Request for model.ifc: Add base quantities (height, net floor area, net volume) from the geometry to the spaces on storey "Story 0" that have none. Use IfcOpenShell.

First a look at what the model holds.

```python
import ifcopenshell
import ifcopenshell.util.element
import ifcopenshell.util.unit

model = ifcopenshell.open("model.ifc")
print(model.schema)
for unit_type in ("LENGTHUNIT", "AREAUNIT", "VOLUMEUNIT"):
    print(unit_type, ifcopenshell.util.unit.calculate_unit_scale(model, unit_type))
storey = next(s for s in model.by_type("IfcBuildingStorey") if s.Name == "Story 0")
spaces = [e for e in ifcopenshell.util.element.get_decomposition(storey) if e.is_a("IfcSpace")]
for e in sorted(spaces, key=lambda e: e.id()):
    print(e.id(), e.is_a(), e.Name, list(ifcopenshell.util.element.get_psets(e, qtos_only=True)), sep=" | ")
```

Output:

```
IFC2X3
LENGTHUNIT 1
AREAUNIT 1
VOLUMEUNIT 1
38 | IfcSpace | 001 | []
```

```python
import ifcopenshell
import ifcopenshell.api.pset
import ifcopenshell.geom
import ifcopenshell.util.element
import ifcopenshell.util.shape
import ifcopenshell.util.unit

model = ifcopenshell.open("model.ifc")
unit_scale = ifcopenshell.util.unit.calculate_unit_scale(model)
area_scale = ifcopenshell.util.unit.calculate_unit_scale(model, "AREAUNIT")
volume_scale = ifcopenshell.util.unit.calculate_unit_scale(model, "VOLUMEUNIT")
settings = ifcopenshell.geom.settings()

storey = next(s for s in model.by_type("IfcBuildingStorey") if s.Name == "Story 0")
spaces = [e for e in ifcopenshell.util.element.get_decomposition(storey) if e.is_a("IfcSpace")]

for e in sorted(spaces, key=lambda e: e.id()):
    if ifcopenshell.util.element.get_psets(e, qtos_only=True, should_inherit=False):
        continue
    # Geometry comes back in metres, in the element's own axes.
    shape = ifcopenshell.geom.create_shape(settings, e)
    values = {
        "Height": ifcopenshell.util.shape.get_z(shape.geometry) / unit_scale,
        "NetFloorArea": ifcopenshell.util.shape.get_footprint_area(shape.geometry) / area_scale,
        "NetVolume": ifcopenshell.util.shape.get_volume(shape.geometry) / volume_scale,
    }
    qto = ifcopenshell.api.pset.add_qto(model, product=e, name="BaseQuantities")
    ifcopenshell.api.pset.edit_qto(model, qto=qto, properties=values)
    print(e.id(), {k: round(v, 3) for k, v in values.items()})

model.write("model-out.ifc")
```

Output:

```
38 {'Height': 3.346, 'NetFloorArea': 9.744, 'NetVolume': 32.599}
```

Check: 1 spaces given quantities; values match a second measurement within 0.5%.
